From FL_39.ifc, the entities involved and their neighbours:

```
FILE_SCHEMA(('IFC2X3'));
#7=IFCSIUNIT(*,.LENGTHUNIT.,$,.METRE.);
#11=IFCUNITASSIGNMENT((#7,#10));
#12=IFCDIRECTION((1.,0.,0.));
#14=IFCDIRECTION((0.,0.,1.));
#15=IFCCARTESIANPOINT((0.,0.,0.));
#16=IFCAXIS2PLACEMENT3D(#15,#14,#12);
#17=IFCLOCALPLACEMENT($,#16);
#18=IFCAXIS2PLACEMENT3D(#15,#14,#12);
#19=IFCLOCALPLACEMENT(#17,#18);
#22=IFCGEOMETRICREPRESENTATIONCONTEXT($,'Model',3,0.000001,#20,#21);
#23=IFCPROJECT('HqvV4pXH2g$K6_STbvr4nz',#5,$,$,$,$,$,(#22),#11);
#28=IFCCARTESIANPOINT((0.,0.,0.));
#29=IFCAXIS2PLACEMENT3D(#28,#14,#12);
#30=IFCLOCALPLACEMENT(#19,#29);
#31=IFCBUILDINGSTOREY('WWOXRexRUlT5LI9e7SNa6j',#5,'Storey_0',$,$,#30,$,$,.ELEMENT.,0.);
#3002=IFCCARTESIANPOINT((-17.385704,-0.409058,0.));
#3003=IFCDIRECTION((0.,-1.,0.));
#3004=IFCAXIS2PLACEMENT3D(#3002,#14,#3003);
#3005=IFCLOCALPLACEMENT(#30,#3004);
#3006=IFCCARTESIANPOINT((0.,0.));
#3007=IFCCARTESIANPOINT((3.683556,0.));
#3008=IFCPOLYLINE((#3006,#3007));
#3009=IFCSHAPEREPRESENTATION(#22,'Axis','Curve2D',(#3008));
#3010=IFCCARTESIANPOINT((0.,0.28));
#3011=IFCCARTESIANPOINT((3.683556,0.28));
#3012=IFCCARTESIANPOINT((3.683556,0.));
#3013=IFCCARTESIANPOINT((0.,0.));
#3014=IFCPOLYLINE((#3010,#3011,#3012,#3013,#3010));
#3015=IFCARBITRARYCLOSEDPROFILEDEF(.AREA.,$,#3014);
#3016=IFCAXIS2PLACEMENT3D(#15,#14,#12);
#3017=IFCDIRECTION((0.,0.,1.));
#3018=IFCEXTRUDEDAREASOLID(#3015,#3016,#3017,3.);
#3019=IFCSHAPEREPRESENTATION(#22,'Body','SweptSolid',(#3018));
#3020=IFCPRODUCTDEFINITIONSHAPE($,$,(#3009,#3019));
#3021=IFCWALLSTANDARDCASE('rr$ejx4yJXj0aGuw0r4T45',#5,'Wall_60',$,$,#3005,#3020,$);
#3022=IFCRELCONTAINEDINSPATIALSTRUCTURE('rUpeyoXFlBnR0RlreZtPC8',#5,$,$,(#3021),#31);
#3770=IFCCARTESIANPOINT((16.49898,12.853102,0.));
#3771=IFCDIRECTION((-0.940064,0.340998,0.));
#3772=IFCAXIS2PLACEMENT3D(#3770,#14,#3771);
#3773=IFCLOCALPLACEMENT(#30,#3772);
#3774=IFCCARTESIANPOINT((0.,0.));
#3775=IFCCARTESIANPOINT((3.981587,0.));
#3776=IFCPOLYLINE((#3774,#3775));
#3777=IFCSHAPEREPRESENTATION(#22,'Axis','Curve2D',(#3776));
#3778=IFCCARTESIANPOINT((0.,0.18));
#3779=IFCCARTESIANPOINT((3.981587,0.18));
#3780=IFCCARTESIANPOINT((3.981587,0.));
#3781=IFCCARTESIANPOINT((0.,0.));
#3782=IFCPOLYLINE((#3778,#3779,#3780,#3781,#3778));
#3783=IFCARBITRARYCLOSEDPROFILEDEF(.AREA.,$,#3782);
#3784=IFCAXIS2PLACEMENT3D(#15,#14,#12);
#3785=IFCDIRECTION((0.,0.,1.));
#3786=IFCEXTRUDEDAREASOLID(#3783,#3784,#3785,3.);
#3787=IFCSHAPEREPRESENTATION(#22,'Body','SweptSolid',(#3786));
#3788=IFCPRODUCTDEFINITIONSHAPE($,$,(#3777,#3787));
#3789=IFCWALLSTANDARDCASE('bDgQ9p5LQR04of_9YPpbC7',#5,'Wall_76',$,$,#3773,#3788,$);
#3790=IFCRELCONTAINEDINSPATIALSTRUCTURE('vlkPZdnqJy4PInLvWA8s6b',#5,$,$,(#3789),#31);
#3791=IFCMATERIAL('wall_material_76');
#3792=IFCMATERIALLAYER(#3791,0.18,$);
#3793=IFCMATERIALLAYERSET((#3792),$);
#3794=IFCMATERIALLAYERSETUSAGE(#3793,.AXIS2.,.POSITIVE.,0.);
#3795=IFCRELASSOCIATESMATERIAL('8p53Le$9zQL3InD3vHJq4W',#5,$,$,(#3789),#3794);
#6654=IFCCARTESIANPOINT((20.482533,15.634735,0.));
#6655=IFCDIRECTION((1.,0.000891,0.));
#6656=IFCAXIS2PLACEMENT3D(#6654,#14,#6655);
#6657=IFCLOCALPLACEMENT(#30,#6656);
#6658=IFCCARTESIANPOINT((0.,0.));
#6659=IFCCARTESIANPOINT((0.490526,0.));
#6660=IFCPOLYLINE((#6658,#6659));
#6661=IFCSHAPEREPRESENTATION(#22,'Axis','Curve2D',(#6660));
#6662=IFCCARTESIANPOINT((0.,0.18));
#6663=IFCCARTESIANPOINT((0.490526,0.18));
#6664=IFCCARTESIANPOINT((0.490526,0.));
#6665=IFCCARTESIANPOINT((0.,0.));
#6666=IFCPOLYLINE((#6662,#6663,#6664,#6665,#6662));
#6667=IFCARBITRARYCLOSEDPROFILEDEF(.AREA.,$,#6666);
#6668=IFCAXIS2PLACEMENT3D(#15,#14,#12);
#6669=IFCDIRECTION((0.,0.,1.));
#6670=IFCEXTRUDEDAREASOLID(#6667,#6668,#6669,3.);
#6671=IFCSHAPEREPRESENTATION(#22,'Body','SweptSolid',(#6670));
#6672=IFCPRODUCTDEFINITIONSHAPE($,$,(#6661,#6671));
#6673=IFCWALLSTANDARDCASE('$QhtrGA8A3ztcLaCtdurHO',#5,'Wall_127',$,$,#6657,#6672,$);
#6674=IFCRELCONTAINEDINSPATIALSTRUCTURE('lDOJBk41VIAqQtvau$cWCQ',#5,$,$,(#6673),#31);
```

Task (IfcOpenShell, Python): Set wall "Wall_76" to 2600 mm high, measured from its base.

```python
import ifcopenshell
import ifcopenshell.geom
import ifcopenshell.util.shape
import ifcopenshell.util.unit

model = ifcopenshell.open("FL_39.ifc")
unit_scale = ifcopenshell.util.unit.calculate_unit_scale(model)
settings = ifcopenshell.geom.settings()


def volume(element):
    """Net volume in cubic metres, openings subtracted."""
    shape = ifcopenshell.geom.create_shape(settings, element)
    return ifcopenshell.util.shape.get_volume(shape.geometry)


wall = model.by_guid("bDgQ9p5LQR04of_9YPpbC7")
before = volume(wall)

body = next(r for r in wall.Representation.Representations if r.RepresentationIdentifier == "Body")
solid = body.Items[0]
old_height = solid.Depth
solid.Depth = 2.6 / unit_scale
after = volume(wall)

print(f"height {old_height:g} -> {solid.Depth:g}, volume {before:.3f} -> {after:.3f} m3")

model.write("FL_39_edited.ifc")
```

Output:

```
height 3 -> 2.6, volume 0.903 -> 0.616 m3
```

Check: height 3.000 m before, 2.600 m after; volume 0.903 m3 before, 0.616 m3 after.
